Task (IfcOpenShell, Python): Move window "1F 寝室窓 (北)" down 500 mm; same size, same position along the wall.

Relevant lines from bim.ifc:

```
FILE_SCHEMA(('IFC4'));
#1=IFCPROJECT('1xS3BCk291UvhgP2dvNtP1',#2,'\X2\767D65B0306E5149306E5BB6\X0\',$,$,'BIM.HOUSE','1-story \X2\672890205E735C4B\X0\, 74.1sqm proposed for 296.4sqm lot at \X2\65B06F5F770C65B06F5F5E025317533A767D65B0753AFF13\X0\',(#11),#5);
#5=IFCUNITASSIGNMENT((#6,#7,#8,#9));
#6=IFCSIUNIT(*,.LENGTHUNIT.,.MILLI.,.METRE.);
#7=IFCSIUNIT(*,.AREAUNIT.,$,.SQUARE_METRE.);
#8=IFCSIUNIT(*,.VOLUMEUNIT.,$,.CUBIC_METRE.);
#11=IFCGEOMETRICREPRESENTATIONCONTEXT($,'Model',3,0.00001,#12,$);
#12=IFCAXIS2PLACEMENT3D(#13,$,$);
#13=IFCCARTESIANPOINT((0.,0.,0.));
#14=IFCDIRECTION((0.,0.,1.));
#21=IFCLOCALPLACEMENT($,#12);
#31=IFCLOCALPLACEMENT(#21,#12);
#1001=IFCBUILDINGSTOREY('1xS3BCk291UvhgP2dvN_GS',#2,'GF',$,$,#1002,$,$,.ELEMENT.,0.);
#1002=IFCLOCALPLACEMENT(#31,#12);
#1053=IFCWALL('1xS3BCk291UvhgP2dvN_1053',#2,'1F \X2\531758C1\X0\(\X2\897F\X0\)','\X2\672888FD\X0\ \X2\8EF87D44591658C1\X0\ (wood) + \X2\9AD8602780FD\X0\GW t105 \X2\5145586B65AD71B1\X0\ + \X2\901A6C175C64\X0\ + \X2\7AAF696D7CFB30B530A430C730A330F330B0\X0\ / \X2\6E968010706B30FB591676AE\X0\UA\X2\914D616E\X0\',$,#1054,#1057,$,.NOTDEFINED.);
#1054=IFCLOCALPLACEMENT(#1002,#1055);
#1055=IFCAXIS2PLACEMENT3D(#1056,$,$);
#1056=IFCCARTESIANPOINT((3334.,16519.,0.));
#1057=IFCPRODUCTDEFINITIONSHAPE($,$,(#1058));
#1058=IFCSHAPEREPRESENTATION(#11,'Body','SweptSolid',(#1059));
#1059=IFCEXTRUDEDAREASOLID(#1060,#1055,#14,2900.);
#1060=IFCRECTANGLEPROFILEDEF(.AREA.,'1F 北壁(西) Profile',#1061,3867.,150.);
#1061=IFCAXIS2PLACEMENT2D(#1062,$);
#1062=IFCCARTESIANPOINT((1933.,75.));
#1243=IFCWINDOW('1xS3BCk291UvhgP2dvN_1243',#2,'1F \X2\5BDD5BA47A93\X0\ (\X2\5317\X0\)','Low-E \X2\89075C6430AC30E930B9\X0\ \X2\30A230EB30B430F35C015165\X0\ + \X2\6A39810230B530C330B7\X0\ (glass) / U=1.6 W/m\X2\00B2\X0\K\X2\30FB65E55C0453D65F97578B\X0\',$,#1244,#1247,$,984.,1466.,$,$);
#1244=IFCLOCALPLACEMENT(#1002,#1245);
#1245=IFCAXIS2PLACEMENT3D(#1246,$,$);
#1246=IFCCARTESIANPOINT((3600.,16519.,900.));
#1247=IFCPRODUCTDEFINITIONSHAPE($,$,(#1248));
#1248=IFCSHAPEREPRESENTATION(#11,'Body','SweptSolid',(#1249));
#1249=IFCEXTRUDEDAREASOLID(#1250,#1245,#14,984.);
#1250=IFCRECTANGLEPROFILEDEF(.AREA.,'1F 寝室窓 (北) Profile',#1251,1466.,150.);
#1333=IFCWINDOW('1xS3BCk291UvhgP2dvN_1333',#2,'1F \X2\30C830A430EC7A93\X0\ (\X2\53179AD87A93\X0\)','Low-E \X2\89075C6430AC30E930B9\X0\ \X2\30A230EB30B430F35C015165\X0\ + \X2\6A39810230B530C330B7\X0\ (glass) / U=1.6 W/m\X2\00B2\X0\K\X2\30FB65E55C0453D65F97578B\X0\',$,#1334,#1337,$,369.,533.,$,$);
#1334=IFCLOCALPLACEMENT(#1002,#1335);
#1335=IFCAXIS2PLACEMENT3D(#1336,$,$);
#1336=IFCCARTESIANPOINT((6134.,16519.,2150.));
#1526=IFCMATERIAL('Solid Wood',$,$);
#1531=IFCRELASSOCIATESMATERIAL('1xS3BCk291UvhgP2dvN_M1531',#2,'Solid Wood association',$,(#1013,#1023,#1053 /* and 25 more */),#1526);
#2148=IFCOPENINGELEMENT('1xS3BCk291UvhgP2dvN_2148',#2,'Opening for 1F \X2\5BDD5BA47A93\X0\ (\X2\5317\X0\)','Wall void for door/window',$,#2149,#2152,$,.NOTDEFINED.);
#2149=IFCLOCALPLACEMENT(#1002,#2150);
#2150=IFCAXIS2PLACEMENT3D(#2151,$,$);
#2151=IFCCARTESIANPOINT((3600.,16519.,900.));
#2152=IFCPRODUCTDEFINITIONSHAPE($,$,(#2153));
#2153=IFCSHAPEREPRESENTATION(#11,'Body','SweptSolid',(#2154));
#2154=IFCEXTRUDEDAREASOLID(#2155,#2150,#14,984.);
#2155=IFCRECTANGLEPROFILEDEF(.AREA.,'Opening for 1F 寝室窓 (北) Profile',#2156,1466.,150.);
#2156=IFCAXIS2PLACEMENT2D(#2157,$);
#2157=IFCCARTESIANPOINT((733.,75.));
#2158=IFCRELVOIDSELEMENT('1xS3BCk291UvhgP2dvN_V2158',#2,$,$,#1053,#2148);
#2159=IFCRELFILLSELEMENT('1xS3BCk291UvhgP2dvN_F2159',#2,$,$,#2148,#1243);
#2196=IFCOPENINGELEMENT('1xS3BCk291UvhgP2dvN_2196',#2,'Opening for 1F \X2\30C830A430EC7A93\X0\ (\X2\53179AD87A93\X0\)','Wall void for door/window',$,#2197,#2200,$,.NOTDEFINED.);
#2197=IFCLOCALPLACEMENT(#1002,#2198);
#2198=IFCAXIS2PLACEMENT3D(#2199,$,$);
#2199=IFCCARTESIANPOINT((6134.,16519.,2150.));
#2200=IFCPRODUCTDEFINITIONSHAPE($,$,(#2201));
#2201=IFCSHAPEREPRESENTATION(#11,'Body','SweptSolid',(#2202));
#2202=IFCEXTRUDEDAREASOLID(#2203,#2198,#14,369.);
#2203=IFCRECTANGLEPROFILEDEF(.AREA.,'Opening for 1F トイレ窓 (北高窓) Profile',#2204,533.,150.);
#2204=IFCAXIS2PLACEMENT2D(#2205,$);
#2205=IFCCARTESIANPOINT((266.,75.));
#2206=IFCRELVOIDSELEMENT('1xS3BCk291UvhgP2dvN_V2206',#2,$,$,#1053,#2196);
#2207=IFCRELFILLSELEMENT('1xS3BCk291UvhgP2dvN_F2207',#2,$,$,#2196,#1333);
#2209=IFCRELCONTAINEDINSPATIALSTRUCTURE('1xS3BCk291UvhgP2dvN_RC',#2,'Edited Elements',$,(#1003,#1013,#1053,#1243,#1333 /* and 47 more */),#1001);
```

```python
import numpy as np
import ifcopenshell
import ifcopenshell.api.geometry
import ifcopenshell.util.placement
import ifcopenshell.util.unit

model = ifcopenshell.open("bim.ifc")
unit_scale = ifcopenshell.util.unit.calculate_unit_scale(model)

window = model.by_guid("1xS3BCk291UvhgP2dvN_1243")
opening = window.FillsVoids[0].RelatingOpeningElement
dz = -500.0

shift = np.array([0.0, 0.0, dz])
# The window is not placed relative to its opening, so move both.
for product in (opening, window):
    matrix = ifcopenshell.util.placement.get_local_placement(product.ObjectPlacement)
    matrix[:3, 3] += shift
    ifcopenshell.api.geometry.edit_object_placement(model, product=product, matrix=matrix, is_si=False)

print(f"moved by {dz * unit_scale:+.3f} m")

model.write("bim_updated.ifc")
```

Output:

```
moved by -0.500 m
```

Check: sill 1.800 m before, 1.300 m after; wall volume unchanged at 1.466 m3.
